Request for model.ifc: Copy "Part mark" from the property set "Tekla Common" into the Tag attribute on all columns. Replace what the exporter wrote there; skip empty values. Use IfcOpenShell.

First a look at what the model holds.

```python
import ifcopenshell
import ifcopenshell.util.element

model = ifcopenshell.open("model.ifc")
print(model.schema)
columns = model.by_type("IfcColumn")
print(len(columns), "columns")
for e in columns[:8]:
    source = ifcopenshell.util.element.get_pset(e, "Tekla Common", "Part mark")
    target = e.Tag
    print(e.id(), repr(source), repr(target), sep=" | ")
```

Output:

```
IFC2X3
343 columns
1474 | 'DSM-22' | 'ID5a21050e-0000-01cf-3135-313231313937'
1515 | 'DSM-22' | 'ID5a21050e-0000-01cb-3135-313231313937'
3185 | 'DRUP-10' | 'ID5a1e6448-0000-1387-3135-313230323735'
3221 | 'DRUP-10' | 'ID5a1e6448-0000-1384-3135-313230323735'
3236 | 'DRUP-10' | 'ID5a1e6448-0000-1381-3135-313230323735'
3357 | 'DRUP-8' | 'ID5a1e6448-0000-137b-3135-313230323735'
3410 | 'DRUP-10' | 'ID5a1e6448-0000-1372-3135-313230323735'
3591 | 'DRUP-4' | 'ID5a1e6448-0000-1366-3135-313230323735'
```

```python
import ifcopenshell
import ifcopenshell.util.element

model = ifcopenshell.open("model.ifc")

count = 0
for e in model.by_type("IfcColumn"):
    value = ifcopenshell.util.element.get_pset(e, "Tekla Common", "Part mark")
    current = e.Tag
    if not value or not value.strip() or current == value:
        continue
    e.Tag = value
    count += 1

print(count, "columns updated")

model.write("model_edited.ifc")
```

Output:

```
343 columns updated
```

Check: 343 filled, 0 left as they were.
